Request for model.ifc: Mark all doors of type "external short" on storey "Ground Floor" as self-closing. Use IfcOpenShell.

First a look at what the model holds.

```python
import ifcopenshell
import ifcopenshell.util.element

model = ifcopenshell.open("model.ifc")
print(model.schema)
storey = next(s for s in model.by_type("IfcBuildingStorey") if s.Name == "Ground Floor")
doors = [e for e in ifcopenshell.util.element.get_decomposition(storey) if e.is_a("IfcDoor")]
seen = {}
for e in doors:
    element_type = ifcopenshell.util.element.get_type(e)
    key = (element_type.Name if element_type != e and element_type else None, ifcopenshell.util.element.get_pset(e, "Pset_DoorCommon", "SelfClosing"))
    seen[key] = seen.get(key, 0) + 1
for (name, value), count in sorted(seen.items(), key=str):
    print(count, "x", name, "|", value)
```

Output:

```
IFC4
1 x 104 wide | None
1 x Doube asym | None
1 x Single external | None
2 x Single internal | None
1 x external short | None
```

```python
import ifcopenshell
import ifcopenshell.api.pset
import ifcopenshell.util.element

model = ifcopenshell.open("model.ifc")

storey = next(s for s in model.by_type("IfcBuildingStorey") if s.Name == "Ground Floor")
doors = [e for e in ifcopenshell.util.element.get_decomposition(storey) if e.is_a("IfcDoor")]

count = 0
for e in doors:
    element_type = ifcopenshell.util.element.get_type(e)
    if element_type in (None, e) or element_type.Name != "external short":
        continue
    # add_pset returns the element's existing set when there is one.
    pset = ifcopenshell.api.pset.add_pset(model, product=e, name="Pset_DoorCommon")
    ifcopenshell.api.pset.edit_pset(model, pset=pset, properties={"SelfClosing": True})
    count += 1

print(count, "doors updated")

model.write("model-out.ifc")
```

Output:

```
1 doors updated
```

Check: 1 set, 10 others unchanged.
